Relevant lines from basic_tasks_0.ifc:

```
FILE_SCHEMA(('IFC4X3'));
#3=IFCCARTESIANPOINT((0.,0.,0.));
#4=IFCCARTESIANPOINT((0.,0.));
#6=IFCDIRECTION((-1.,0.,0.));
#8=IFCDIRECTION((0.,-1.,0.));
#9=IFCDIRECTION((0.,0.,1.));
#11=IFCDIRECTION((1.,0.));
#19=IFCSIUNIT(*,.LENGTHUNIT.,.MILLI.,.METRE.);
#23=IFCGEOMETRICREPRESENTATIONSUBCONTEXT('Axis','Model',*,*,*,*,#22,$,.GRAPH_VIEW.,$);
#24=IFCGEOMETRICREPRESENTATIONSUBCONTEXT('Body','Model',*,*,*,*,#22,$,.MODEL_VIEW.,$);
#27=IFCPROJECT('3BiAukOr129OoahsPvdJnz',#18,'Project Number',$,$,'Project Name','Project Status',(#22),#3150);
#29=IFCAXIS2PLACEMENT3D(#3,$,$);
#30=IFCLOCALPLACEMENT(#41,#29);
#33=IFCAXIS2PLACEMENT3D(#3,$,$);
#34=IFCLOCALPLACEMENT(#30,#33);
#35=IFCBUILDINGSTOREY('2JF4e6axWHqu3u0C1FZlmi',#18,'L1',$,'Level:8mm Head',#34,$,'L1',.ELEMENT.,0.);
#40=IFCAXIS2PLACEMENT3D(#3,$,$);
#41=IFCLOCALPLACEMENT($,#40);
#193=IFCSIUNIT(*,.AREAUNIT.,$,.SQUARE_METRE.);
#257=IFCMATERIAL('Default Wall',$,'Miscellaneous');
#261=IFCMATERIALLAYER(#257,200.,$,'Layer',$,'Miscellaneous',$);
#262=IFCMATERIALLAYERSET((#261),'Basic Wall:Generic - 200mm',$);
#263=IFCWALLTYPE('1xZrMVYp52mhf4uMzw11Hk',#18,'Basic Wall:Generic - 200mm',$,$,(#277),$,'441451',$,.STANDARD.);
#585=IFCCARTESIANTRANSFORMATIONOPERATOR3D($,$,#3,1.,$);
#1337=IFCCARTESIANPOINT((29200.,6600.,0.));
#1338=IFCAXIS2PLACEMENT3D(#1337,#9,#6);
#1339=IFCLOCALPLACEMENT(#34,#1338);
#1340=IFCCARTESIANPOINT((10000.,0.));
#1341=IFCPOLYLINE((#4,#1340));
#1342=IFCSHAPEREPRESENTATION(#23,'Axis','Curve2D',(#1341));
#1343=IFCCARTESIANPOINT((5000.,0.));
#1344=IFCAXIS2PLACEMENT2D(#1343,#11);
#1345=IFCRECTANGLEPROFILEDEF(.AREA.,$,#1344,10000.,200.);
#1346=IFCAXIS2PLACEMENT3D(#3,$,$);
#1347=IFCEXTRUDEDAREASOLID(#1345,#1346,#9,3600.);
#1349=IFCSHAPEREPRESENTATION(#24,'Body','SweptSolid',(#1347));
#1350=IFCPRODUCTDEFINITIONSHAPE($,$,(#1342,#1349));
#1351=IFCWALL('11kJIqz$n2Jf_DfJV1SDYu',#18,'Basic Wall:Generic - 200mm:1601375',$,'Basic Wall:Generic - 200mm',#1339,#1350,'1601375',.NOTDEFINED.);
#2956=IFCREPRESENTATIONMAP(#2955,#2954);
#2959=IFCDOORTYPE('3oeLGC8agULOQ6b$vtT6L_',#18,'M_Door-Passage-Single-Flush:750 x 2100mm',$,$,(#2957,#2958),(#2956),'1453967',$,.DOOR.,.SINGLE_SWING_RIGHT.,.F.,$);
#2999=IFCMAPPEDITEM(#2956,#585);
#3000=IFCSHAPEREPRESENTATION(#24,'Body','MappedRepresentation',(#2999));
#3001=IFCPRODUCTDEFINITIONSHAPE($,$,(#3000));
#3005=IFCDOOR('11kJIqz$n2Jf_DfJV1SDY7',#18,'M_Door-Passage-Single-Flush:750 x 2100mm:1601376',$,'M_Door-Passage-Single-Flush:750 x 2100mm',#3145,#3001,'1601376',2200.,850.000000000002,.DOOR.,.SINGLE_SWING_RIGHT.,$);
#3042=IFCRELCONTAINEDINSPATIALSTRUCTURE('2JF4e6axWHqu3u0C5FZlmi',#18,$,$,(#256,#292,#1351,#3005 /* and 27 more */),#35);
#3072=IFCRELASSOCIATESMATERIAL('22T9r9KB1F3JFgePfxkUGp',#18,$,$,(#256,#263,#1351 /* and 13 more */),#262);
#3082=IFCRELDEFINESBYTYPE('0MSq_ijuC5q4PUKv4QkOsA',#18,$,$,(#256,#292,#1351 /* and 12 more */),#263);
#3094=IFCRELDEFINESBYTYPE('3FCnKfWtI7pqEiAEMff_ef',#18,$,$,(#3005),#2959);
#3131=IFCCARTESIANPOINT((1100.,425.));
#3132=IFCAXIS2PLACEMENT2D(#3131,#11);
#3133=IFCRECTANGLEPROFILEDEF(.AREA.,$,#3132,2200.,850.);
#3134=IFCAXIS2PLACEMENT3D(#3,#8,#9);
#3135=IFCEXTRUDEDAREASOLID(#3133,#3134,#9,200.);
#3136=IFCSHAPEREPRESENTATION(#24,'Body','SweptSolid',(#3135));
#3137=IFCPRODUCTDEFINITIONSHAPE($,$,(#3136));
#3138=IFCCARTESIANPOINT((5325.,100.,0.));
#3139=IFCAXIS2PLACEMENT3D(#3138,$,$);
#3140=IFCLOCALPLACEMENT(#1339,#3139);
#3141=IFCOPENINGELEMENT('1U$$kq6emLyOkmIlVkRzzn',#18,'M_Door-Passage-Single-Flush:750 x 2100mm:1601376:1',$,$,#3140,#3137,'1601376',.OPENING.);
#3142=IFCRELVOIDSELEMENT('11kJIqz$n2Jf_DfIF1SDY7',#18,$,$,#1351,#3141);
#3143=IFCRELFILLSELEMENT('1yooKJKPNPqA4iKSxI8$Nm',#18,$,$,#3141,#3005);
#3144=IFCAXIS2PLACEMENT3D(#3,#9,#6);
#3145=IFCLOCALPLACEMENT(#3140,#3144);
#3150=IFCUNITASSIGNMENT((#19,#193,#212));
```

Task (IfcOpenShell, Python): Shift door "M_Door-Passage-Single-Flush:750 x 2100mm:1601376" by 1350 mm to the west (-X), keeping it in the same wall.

```python
import ifcopenshell
import ifcopenshell.api.geometry
import ifcopenshell.util.placement

model = ifcopenshell.open("basic_tasks_0.ifc")

door = model.by_guid("11kJIqz$n2Jf_DfJV1SDY7")
opening = door.FillsVoids[0].RelatingOpeningElement
wall = opening.VoidsElements[0].RelatingBuildingElement

wall_matrix = ifcopenshell.util.placement.get_local_placement(wall.ObjectPlacement)
shift = wall_matrix[:3, 0] * 1350.0
before = ifcopenshell.util.placement.get_local_placement(door.ObjectPlacement)[:3, 3].copy()

# The door is placed relative to its opening, so it follows when the opening moves.
matrix = ifcopenshell.util.placement.get_local_placement(opening.ObjectPlacement)
matrix[:3, 3] += shift
ifcopenshell.api.geometry.edit_object_placement(
    model, product=opening, matrix=matrix, is_si=False, should_transform_children=True
)

after = ifcopenshell.util.placement.get_local_placement(door.ObjectPlacement)[:3, 3]
print("door moved by", (after - before).round(3) + 0.0)

model.write("basic_tasks_0-out.ifc")
```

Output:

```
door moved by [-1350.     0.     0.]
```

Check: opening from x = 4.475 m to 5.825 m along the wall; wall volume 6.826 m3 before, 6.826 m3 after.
